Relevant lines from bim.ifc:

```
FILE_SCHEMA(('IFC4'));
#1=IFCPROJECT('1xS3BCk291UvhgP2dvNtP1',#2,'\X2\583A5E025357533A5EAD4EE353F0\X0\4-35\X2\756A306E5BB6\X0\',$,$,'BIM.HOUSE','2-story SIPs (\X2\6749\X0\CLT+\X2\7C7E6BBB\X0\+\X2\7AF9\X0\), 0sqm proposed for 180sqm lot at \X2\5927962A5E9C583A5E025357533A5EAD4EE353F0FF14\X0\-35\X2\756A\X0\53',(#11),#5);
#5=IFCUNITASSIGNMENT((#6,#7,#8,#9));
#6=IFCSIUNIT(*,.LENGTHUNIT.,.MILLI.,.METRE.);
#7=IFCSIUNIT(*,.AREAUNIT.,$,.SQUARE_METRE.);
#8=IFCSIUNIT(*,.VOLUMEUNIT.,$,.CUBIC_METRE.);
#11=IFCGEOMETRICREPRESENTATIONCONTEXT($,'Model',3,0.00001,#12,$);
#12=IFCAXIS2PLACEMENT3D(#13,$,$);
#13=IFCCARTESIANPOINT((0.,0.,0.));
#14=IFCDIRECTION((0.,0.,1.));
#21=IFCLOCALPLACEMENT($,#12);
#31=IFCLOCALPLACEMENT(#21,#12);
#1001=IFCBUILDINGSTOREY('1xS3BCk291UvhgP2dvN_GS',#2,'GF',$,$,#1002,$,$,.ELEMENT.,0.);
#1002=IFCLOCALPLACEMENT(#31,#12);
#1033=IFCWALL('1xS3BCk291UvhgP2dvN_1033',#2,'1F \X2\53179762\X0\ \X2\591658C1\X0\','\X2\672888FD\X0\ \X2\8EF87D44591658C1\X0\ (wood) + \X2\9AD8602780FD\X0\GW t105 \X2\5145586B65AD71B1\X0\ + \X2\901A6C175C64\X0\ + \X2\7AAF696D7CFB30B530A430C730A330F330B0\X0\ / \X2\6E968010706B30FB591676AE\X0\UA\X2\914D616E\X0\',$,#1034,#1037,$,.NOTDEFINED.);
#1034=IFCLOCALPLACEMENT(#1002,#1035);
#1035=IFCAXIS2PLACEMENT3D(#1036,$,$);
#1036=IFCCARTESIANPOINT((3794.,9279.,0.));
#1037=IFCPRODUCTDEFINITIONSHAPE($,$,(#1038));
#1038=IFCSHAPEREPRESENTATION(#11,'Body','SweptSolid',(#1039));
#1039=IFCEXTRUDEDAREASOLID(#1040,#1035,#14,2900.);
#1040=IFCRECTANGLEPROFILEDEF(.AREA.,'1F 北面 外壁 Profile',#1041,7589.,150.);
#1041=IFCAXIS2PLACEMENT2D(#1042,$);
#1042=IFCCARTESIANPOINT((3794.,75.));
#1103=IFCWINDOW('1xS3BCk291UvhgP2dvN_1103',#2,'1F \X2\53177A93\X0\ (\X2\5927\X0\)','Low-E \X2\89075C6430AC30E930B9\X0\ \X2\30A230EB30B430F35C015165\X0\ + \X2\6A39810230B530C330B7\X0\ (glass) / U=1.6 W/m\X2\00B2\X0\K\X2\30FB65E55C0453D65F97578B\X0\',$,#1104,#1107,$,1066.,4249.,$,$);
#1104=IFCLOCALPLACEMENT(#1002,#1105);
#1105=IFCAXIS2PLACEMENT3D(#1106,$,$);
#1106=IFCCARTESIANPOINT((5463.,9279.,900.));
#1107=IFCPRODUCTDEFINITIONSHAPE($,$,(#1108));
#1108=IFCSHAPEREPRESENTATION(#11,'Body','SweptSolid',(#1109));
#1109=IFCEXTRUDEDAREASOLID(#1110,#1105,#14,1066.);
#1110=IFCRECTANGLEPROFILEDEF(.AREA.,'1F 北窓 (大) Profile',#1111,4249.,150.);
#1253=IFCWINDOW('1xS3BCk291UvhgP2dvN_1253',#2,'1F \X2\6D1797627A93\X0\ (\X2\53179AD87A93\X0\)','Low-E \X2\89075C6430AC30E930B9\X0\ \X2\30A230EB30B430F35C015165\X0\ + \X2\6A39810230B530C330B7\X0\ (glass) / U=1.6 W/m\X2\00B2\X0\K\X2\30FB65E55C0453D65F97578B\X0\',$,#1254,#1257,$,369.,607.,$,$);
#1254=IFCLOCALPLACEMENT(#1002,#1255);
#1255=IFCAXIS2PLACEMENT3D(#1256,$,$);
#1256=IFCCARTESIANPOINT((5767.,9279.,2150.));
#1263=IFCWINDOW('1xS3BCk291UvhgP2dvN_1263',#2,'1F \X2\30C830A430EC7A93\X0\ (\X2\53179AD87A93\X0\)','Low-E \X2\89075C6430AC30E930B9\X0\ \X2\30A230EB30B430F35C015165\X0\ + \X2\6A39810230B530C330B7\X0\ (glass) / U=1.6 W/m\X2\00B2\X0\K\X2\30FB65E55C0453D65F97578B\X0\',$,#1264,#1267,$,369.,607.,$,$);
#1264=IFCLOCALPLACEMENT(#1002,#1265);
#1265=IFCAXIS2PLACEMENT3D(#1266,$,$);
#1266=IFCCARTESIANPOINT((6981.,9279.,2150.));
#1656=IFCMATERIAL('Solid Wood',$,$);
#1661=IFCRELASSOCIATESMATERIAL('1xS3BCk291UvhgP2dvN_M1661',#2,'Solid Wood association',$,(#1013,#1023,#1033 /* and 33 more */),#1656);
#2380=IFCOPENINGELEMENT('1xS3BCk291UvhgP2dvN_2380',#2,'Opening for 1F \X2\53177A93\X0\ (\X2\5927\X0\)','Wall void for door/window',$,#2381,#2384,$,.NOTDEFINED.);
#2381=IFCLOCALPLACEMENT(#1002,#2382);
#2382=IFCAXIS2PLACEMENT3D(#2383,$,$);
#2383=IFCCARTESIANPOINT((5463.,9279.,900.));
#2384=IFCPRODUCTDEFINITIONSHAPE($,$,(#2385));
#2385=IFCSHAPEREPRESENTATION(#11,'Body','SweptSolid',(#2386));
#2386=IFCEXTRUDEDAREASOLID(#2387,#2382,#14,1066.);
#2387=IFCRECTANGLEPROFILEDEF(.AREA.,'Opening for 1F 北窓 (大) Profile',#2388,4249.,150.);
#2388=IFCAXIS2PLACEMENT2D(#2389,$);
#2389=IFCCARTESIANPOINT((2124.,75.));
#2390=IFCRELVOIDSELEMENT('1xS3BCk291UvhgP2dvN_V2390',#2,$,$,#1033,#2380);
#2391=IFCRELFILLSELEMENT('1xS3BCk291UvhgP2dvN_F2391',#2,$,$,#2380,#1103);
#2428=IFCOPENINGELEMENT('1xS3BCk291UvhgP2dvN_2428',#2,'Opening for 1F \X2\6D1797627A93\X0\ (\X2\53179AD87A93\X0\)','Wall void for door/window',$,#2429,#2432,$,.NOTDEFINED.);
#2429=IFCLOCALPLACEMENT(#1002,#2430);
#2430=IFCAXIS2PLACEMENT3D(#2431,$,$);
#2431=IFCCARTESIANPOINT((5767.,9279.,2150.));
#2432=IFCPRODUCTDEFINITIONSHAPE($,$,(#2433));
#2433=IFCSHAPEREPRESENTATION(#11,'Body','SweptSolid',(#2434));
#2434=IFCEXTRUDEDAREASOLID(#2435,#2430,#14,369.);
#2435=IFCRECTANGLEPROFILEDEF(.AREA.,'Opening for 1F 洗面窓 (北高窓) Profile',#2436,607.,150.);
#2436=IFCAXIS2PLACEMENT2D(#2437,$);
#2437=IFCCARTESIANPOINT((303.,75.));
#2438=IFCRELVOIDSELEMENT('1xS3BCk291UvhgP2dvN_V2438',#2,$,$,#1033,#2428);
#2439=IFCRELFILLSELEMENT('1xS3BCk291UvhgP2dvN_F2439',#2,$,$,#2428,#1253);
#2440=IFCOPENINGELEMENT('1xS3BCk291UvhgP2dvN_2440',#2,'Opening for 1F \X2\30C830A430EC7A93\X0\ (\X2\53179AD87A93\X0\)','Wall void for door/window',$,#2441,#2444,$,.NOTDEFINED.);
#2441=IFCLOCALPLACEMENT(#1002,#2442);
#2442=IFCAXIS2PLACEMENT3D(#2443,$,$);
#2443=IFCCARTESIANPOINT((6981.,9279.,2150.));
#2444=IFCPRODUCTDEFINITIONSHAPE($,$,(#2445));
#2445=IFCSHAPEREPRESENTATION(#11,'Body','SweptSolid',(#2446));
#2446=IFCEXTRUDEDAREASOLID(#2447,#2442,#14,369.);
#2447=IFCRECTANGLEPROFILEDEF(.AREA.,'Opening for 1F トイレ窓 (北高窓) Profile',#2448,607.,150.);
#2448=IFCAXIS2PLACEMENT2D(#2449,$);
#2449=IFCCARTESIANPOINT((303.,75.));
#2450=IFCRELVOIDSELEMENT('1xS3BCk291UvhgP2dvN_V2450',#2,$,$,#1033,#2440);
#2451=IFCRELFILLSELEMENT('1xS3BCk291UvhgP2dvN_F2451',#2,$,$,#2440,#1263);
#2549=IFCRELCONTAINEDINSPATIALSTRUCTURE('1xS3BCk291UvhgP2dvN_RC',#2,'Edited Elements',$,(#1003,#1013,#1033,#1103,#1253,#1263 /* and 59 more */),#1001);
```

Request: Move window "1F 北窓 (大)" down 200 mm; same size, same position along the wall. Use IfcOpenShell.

```python
import numpy as np
import ifcopenshell
import ifcopenshell.api.geometry
import ifcopenshell.util.placement
import ifcopenshell.util.unit

model = ifcopenshell.open("bim.ifc")
unit_scale = ifcopenshell.util.unit.calculate_unit_scale(model)

window = model.by_guid("1xS3BCk291UvhgP2dvN_1103")
opening = window.FillsVoids[0].RelatingOpeningElement
dz = -0.2 / unit_scale

shift = np.array([0.0, 0.0, dz])
# The window is not placed relative to its opening, so move both.
for product in (opening, window):
    matrix = ifcopenshell.util.placement.get_local_placement(product.ObjectPlacement)
    matrix[:3, 3] += shift
    ifcopenshell.api.geometry.edit_object_placement(model, product=product, matrix=matrix, is_si=False)

print(f"moved by {dz * unit_scale:+.3f} m")

model.write("bim_updated.ifc")
```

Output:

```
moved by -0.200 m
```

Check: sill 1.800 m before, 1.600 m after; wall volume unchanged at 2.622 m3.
